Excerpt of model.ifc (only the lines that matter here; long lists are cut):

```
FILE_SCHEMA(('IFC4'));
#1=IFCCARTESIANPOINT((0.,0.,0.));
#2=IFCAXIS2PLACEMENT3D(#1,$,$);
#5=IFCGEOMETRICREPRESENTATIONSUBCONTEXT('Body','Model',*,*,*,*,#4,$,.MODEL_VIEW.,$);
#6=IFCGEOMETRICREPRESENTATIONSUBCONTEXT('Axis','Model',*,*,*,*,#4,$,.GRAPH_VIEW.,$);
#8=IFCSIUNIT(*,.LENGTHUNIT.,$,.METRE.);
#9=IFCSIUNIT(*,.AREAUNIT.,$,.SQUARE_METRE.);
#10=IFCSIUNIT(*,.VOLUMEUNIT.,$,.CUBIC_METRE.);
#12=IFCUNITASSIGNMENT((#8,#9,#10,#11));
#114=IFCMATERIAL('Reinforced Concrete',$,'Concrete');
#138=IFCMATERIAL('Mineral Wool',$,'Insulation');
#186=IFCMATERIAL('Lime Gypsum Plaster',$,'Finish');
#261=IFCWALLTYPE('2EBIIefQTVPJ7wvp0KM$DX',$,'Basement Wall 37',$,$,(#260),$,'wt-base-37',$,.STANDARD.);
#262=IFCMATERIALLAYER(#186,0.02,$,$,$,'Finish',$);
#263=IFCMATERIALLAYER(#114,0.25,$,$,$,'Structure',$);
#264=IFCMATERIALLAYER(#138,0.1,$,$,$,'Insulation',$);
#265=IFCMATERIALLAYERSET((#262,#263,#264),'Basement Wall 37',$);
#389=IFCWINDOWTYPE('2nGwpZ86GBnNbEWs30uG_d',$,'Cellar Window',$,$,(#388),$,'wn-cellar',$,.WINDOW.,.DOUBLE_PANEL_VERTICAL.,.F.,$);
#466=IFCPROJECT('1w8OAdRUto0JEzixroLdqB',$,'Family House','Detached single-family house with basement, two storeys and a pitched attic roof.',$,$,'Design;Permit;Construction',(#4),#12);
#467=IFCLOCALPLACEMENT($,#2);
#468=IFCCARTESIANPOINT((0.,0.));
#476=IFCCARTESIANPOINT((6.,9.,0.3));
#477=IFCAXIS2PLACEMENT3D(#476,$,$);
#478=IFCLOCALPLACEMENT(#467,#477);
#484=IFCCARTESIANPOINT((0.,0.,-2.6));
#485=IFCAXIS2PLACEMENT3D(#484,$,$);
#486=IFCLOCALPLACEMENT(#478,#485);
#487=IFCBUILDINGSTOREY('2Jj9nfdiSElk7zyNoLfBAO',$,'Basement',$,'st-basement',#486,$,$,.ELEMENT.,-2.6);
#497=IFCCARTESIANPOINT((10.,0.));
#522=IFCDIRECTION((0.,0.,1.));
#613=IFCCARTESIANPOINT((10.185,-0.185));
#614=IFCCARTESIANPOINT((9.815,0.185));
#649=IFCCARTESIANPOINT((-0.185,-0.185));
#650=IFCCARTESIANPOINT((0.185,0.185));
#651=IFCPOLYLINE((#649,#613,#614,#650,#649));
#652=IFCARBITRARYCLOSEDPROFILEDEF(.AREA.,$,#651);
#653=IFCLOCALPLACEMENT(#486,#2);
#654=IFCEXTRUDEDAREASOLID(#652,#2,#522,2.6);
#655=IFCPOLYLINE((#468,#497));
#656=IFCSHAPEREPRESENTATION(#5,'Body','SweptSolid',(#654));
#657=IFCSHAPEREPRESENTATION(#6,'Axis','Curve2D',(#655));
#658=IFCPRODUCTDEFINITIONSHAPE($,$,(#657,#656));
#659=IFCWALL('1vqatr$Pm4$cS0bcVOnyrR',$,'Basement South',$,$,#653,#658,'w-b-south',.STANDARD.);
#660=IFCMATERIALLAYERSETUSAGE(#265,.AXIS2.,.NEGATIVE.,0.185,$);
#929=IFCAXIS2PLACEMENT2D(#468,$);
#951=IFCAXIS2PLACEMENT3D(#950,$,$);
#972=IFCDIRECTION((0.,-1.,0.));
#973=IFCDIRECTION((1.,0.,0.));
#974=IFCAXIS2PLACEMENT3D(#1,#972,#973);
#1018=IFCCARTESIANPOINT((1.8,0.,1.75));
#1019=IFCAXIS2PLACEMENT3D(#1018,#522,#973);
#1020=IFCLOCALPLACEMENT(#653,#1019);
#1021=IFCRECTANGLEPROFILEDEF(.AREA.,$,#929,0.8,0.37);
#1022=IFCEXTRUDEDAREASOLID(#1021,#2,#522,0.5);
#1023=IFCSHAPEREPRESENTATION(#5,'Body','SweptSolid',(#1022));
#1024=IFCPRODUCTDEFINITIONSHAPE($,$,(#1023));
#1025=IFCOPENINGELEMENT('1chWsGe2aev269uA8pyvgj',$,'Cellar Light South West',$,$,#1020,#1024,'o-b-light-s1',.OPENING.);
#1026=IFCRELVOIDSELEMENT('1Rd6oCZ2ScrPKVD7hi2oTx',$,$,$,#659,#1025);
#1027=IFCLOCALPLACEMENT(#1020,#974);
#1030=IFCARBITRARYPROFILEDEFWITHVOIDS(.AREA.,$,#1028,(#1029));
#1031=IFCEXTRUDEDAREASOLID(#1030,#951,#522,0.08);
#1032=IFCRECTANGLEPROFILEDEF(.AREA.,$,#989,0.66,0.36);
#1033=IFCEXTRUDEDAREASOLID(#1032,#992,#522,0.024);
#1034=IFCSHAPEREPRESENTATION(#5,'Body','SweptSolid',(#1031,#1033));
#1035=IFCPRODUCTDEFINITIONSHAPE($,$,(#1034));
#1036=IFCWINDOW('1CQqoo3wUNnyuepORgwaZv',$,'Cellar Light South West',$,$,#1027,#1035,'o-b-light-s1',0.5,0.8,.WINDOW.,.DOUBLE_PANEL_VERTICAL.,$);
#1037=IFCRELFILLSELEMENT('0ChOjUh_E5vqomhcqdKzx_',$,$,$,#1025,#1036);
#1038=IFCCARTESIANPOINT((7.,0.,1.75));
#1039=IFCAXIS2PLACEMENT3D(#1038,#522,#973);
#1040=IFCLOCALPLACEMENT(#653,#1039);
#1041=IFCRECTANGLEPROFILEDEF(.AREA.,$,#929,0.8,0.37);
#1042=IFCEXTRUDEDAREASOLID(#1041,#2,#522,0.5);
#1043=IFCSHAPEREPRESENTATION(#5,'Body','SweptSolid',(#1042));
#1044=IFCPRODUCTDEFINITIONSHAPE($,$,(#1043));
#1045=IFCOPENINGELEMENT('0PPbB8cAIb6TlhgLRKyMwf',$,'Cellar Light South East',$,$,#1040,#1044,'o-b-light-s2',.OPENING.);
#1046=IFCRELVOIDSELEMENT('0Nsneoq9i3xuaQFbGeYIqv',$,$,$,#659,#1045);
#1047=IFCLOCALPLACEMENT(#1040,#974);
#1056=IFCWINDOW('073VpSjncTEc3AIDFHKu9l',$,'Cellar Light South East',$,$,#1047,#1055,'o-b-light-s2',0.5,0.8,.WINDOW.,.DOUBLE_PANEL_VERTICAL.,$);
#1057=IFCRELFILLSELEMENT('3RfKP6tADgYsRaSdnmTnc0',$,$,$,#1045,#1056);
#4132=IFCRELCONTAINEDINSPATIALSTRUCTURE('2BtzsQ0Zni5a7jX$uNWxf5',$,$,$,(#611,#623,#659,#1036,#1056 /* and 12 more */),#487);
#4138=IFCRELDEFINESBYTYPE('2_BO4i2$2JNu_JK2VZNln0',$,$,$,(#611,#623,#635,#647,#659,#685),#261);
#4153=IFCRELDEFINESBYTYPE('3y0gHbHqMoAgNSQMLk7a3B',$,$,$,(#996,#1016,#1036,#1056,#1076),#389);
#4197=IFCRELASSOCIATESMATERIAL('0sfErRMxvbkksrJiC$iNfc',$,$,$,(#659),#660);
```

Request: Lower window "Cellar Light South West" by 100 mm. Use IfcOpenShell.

```python
import numpy as np
import ifcopenshell
import ifcopenshell.api.geometry
import ifcopenshell.util.placement
import ifcopenshell.util.unit

model = ifcopenshell.open("model.ifc")
unit_scale = ifcopenshell.util.unit.calculate_unit_scale(model)

window = model.by_guid("1CQqoo3wUNnyuepORgwaZv")
opening = window.FillsVoids[0].RelatingOpeningElement
dz = -0.1

shift = np.array([0.0, 0.0, dz])
# The window is placed relative to its opening, so it follows when the opening moves.
matrix = ifcopenshell.util.placement.get_local_placement(opening.ObjectPlacement)
matrix[:3, 3] += shift
ifcopenshell.api.geometry.edit_object_placement(
    model, product=opening, matrix=matrix, is_si=False, should_transform_children=True
)

print(f"moved by {dz * unit_scale:+.3f} m")

model.write("model-out.ifc")
```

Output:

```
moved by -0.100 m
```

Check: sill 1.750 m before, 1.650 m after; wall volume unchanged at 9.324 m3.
